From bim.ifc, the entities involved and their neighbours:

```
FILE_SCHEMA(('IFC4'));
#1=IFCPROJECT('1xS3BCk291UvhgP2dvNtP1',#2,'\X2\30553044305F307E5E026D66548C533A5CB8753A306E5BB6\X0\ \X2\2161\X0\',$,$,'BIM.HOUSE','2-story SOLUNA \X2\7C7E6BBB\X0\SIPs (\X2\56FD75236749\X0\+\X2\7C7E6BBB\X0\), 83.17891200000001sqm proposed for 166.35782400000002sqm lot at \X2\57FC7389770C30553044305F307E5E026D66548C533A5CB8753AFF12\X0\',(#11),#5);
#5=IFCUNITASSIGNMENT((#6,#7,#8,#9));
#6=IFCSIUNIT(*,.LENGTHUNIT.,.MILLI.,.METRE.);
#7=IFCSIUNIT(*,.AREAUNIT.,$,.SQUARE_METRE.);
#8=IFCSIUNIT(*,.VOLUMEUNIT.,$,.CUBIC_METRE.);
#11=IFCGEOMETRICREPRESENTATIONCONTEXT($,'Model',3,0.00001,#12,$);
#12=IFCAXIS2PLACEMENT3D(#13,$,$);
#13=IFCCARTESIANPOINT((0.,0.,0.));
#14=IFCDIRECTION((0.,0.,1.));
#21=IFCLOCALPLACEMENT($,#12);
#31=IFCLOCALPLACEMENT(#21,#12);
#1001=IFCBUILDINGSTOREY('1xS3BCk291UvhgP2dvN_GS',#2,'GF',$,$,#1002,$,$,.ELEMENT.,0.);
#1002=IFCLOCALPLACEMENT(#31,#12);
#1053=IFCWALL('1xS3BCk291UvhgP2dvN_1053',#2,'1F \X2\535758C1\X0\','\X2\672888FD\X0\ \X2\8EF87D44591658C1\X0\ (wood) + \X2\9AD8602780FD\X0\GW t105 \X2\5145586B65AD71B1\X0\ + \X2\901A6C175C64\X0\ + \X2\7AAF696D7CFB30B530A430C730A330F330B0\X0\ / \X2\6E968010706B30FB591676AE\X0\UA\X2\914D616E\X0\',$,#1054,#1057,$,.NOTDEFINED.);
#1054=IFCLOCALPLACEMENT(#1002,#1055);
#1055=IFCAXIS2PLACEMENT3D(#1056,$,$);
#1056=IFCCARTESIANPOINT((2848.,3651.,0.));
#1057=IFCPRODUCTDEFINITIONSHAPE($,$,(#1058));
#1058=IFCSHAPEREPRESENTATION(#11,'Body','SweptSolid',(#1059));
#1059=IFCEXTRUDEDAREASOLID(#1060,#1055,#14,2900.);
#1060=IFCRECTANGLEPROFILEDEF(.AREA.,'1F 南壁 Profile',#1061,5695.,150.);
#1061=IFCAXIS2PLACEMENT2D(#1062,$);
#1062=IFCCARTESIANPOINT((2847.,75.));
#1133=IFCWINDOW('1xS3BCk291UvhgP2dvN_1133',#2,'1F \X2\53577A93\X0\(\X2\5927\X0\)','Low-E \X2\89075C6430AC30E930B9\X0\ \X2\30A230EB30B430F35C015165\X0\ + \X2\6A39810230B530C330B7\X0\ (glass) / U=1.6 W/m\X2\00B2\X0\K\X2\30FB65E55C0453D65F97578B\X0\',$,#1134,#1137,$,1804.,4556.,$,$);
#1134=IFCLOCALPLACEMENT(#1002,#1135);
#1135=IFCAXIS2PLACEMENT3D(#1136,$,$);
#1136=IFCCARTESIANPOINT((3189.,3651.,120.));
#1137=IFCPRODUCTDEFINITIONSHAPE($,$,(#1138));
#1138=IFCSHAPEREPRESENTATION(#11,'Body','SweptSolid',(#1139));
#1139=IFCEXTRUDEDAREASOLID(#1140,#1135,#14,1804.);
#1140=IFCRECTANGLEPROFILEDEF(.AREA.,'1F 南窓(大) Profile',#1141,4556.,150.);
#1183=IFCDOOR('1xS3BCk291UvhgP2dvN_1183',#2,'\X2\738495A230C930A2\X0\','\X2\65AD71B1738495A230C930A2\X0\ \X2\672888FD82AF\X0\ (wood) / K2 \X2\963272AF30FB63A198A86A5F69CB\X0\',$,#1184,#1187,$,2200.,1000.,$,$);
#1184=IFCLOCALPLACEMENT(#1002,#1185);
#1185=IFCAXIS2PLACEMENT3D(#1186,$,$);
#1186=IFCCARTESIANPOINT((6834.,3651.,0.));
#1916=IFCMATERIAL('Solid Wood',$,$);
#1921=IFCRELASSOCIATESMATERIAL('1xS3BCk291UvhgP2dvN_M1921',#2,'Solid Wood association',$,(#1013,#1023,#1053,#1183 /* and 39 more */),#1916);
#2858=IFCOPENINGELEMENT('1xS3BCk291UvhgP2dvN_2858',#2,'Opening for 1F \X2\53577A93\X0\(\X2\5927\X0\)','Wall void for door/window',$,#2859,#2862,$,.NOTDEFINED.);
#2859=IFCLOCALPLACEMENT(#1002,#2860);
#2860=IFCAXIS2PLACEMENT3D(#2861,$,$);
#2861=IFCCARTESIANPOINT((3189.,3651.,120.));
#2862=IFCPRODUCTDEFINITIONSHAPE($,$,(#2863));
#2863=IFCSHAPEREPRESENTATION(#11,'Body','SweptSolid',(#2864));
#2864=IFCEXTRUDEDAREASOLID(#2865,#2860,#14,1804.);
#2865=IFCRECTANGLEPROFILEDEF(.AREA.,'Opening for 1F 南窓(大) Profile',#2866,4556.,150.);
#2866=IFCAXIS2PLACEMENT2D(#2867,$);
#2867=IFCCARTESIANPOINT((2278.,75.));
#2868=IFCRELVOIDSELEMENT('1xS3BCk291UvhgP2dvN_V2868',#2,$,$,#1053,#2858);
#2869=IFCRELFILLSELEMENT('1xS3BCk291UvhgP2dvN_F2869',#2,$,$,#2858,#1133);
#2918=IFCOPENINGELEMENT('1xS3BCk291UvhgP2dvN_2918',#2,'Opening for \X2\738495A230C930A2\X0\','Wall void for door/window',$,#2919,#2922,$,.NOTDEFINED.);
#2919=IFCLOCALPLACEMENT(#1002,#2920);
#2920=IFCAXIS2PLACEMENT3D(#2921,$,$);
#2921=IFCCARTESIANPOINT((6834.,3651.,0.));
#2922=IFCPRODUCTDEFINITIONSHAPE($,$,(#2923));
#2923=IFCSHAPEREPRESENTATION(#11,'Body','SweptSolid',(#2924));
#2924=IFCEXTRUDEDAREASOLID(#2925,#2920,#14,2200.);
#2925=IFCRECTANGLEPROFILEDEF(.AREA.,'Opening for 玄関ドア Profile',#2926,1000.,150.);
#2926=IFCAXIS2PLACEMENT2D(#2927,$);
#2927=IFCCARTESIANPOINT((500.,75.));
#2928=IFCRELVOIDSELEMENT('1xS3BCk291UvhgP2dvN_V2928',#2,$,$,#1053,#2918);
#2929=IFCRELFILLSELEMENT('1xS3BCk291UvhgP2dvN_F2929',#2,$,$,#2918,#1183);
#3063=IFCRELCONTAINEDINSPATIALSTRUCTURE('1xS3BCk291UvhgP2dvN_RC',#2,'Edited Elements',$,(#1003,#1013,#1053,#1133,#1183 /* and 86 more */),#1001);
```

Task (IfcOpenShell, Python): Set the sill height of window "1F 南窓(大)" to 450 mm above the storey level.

```python
import numpy as np
import ifcopenshell
import ifcopenshell.api.geometry
import ifcopenshell.geom
import ifcopenshell.util.element
import ifcopenshell.util.placement
import ifcopenshell.util.shape
import ifcopenshell.util.unit

model = ifcopenshell.open("bim.ifc")
unit_scale = ifcopenshell.util.unit.calculate_unit_scale(model)

window = model.by_guid("1xS3BCk291UvhgP2dvN_1133")
opening = window.FillsVoids[0].RelatingOpeningElement
storey = ifcopenshell.util.element.get_container(window, ifc_class="IfcBuildingStorey")
level = ifcopenshell.util.placement.get_local_placement(storey.ObjectPlacement)[2, 3]

# The opening's origin need not be at the sill, so measure its lowest point.
shape = ifcopenshell.geom.create_shape(ifcopenshell.geom.settings(), opening)
bottom = ifcopenshell.util.shape.get_shape_bottom_elevation(shape, shape.geometry) / unit_scale
dz = level + 0.45 / unit_scale - bottom

shift = np.array([0.0, 0.0, dz])
# The window is not placed relative to its opening, so move both.
for product in (opening, window):
    matrix = ifcopenshell.util.placement.get_local_placement(product.ObjectPlacement)
    matrix[:3, 3] += shift
    ifcopenshell.api.geometry.edit_object_placement(model, product=product, matrix=matrix, is_si=False)

print(f"moved by {dz * unit_scale:+.3f} m")

model.write("bim_edited.ifc")
```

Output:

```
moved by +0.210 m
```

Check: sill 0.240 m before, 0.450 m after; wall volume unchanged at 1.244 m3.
